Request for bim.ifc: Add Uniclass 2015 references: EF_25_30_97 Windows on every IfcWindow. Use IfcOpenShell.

First a look at what the model holds.

```python
import ifcopenshell

model = ifcopenshell.open("bim.ifc")
print(model.schema)
print("classifications:", [c.Name for c in model.by_type("IfcClassification")])
for ifc_class in ("IfcDoor", "IfcRoof", "IfcStair", "IfcWall", "IfcWindow"):
    print(ifc_class, len(model.by_type(ifc_class)))
```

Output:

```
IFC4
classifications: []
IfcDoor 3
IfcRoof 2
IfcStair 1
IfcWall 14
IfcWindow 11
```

```python
import ifcopenshell
import ifcopenshell.api.classification

model = ifcopenshell.open("bim.ifc")

system = ifcopenshell.api.classification.add_classification(model, classification="Uniclass 2015")

codes = {
    "IfcWindow": ("EF_25_30_97", "Windows"),
}
for ifc_class, (code, name) in codes.items():
    products = model.by_type(ifc_class)
    ifcopenshell.api.classification.add_reference(
        model, products=products, classification=system, identification=code, name=name
    )
    print(code, len(products))

model.write("bim_edited.ifc")
```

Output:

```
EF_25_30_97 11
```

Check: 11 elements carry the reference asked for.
